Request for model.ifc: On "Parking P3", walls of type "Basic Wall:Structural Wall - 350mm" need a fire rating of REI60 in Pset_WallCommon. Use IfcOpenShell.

First a look at what the model holds.

```python
import ifcopenshell
import ifcopenshell.util.element

model = ifcopenshell.open("model.ifc")
print(model.schema)
storey = next(s for s in model.by_type("IfcBuildingStorey") if s.Name == "Parking P3")
walls = [e for e in ifcopenshell.util.element.get_decomposition(storey) if e.is_a("IfcWall")]
seen = {}
for e in walls:
    element_type = ifcopenshell.util.element.get_type(e)
    key = (element_type.Name if element_type != e and element_type else None, ifcopenshell.util.element.get_pset(e, "Pset_WallCommon", "FireRating"))
    seen[key] = seen.get(key, 0) + 1
for (name, value), count in sorted(seen.items(), key=str):
    print(count, "x", name, "|", value)
```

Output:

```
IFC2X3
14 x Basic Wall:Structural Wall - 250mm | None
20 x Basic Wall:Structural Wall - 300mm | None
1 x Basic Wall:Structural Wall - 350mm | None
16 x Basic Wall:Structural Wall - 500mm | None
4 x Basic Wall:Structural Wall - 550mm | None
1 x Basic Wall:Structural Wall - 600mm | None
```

```python
import ifcopenshell
import ifcopenshell.api.pset
import ifcopenshell.util.element

model = ifcopenshell.open("model.ifc")

storey = next(s for s in model.by_type("IfcBuildingStorey") if s.Name == "Parking P3")
walls = [e for e in ifcopenshell.util.element.get_decomposition(storey) if e.is_a("IfcWall")]

count = 0
for e in walls:
    element_type = ifcopenshell.util.element.get_type(e)
    if element_type in (None, e) or element_type.Name != "Basic Wall:Structural Wall - 350mm":
        continue
    # add_pset returns the element's existing set when there is one.
    pset = ifcopenshell.api.pset.add_pset(model, product=e, name="Pset_WallCommon")
    ifcopenshell.api.pset.edit_pset(model, pset=pset, properties={"FireRating": "REI60"})
    count += 1

print(count, "walls updated")

model.write("model-out.ifc")
```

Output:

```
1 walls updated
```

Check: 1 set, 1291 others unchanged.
